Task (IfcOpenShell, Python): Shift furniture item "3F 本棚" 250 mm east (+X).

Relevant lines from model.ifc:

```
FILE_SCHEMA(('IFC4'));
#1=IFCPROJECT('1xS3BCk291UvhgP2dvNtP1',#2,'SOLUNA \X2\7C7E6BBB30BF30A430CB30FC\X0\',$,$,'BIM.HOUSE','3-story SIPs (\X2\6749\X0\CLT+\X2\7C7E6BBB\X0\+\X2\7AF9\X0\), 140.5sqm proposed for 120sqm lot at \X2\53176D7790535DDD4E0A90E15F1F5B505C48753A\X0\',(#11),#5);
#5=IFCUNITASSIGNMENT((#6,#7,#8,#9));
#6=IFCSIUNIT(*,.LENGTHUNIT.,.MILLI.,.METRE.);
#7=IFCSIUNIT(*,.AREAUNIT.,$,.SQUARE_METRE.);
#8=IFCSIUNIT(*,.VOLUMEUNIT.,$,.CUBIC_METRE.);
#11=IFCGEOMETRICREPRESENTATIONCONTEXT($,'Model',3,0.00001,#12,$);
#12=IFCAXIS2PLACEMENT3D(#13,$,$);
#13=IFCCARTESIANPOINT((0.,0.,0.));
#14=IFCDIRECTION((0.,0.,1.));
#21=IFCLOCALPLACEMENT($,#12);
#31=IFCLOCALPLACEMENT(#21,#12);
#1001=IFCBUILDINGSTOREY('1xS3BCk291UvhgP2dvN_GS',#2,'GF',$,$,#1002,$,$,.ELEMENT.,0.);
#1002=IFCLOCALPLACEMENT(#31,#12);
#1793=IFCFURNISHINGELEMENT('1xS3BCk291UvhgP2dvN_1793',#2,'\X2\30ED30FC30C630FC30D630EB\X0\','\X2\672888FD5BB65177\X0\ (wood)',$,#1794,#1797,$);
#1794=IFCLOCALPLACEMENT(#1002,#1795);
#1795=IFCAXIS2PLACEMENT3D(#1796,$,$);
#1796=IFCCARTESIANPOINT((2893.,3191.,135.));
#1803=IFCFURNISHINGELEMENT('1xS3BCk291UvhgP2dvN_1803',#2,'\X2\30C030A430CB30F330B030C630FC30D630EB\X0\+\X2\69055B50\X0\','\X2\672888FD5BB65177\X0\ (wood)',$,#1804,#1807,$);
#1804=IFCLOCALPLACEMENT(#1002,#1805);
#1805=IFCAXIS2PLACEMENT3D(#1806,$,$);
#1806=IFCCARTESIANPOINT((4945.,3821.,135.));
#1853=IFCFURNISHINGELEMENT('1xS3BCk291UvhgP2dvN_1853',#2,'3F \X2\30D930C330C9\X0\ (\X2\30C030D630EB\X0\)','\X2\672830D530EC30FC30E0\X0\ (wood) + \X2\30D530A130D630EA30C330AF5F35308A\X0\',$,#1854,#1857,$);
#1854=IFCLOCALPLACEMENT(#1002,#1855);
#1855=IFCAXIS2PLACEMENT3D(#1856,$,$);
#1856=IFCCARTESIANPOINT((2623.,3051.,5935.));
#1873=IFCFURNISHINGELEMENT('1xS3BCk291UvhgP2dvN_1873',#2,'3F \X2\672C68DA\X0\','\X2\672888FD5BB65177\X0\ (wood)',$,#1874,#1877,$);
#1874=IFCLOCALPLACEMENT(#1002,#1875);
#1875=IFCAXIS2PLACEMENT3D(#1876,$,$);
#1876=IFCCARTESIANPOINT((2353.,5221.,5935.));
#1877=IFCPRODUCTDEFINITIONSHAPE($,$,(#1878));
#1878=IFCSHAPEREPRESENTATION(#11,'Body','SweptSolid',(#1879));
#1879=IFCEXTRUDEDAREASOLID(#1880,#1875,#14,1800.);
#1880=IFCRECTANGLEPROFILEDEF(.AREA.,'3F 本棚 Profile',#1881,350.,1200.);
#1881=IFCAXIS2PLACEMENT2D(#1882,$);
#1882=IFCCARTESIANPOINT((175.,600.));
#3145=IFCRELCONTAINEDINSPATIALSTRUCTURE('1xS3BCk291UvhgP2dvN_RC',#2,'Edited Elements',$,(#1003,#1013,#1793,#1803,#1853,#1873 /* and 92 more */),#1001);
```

```python
import ifcopenshell
import ifcopenshell.api.geometry
import ifcopenshell.util.placement

model = ifcopenshell.open("model.ifc")

item = model.by_id(1873)
matrix = ifcopenshell.util.placement.get_local_placement(item.ObjectPlacement)
matrix[0, 3] += 250.0
ifcopenshell.api.geometry.edit_object_placement(model, product=item, matrix=matrix, is_si=False)

print(ifcopenshell.util.placement.get_local_placement(item.ObjectPlacement).round(3) + 0.0)

model.write("model_v2.ifc")
```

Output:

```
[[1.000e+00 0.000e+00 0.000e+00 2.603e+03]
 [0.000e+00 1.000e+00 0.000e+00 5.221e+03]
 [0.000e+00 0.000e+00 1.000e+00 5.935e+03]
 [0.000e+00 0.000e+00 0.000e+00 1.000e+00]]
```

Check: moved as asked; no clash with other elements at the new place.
